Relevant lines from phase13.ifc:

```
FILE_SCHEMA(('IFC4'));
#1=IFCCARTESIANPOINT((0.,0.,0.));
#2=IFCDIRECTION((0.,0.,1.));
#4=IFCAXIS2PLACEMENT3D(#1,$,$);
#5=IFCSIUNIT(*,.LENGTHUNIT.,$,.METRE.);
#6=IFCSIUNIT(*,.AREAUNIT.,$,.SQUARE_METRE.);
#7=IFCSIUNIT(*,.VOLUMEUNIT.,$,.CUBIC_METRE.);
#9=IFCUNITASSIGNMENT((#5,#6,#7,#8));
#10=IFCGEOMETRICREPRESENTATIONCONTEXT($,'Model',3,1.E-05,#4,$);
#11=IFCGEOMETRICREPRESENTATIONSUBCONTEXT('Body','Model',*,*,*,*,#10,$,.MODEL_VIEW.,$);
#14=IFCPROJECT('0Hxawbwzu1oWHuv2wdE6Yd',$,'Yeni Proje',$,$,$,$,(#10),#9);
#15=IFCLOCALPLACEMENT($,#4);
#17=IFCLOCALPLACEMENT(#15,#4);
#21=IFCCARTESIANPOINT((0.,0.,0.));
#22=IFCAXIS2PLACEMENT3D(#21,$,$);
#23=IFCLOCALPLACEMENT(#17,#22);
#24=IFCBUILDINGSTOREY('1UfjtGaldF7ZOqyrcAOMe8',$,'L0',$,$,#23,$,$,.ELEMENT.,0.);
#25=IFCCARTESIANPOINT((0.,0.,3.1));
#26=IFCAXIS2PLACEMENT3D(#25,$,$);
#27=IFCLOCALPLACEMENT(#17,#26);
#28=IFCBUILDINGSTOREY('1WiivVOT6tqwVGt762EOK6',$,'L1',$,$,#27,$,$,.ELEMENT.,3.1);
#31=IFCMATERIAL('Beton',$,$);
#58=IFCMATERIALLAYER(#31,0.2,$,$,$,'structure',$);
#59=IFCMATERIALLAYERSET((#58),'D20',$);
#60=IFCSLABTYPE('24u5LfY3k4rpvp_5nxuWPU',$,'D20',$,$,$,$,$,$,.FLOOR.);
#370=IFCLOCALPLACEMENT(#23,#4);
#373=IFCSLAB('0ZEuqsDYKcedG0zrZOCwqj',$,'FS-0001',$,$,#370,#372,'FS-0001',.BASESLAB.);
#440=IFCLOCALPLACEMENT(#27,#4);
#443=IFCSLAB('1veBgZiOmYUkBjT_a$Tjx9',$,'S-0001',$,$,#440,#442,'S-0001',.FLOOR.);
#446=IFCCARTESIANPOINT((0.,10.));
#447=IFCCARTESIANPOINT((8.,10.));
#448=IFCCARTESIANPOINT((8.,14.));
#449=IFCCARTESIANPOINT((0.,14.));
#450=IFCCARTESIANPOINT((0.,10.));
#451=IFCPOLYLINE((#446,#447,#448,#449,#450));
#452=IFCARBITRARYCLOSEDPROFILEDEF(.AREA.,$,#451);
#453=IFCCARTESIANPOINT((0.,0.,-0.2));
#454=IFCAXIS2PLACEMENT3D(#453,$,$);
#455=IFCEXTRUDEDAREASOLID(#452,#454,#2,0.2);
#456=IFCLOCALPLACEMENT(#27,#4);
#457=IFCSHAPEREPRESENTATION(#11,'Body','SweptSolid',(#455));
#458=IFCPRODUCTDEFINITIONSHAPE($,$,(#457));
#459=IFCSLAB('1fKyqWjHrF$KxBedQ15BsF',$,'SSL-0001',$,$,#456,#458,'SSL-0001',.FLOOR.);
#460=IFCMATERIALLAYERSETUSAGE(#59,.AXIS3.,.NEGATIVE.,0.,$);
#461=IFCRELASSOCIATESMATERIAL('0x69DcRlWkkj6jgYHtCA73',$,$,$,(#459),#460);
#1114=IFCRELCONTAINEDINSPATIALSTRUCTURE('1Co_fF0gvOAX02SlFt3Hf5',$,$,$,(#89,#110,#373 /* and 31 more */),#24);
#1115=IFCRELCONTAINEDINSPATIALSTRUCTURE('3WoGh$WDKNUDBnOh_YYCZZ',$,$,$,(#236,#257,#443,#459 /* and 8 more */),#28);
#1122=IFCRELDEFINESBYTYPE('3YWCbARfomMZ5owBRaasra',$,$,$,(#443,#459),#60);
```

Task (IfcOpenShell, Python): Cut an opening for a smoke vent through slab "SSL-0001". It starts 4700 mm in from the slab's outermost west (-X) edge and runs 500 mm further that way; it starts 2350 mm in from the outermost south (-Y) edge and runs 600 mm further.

```python
import numpy as np
import ifcopenshell
import ifcopenshell.api.feature
import ifcopenshell.api.geometry
import ifcopenshell.api.root
import ifcopenshell.geom
import ifcopenshell.util.placement
import ifcopenshell.util.representation
import ifcopenshell.util.shape
import ifcopenshell.util.unit

model = ifcopenshell.open("phase13.ifc")
unit_scale = ifcopenshell.util.unit.calculate_unit_scale(model)
settings = ifcopenshell.geom.settings()


def volume(element):
    """Net volume in cubic metres, openings subtracted."""
    shape = ifcopenshell.geom.create_shape(settings, element)
    return ifcopenshell.util.shape.get_volume(shape.geometry)


slab = model.by_guid("1fKyqWjHrF$KxBedQ15BsF")
before = volume(slab)

# Extent in the slab's own axes, in metres. The edges named are its -X and -Y sides.
slab_shape = ifcopenshell.geom.create_shape(settings, slab)
vertices = ifcopenshell.util.shape.get_vertices(slab_shape.geometry)
x_min, y_min, bottom = vertices.min(axis=0)
top = vertices[:, 2].max()

opening = ifcopenshell.api.root.create_entity(model, ifc_class="IfcOpeningElement", name="Smoke vent opening", predefined_type="OPENING")
context = ifcopenshell.util.representation.get_context(model, "Model", "Body", "MODEL_VIEW")
width, depth = 0.5, 0.6
outline = [(0.0, 0.0), (width, 0.0), (width, depth), (0.0, depth), (0.0, 0.0)]
# Overshoot both faces by 50 mm so the cut is clean.
shape = ifcopenshell.api.geometry.add_slab_representation(
    model, context=context, depth=top - bottom + 0.1, polyline=outline
)
ifcopenshell.api.geometry.assign_representation(model, product=opening, representation=shape)

matrix = ifcopenshell.util.placement.get_local_placement(slab.ObjectPlacement)
matrix[:, 3] = matrix @ np.append(np.array([x_min + 4.7, y_min + 2.35, bottom - 0.05]) / unit_scale, 1.0)
ifcopenshell.api.geometry.edit_object_placement(model, product=opening, matrix=matrix, is_si=False)
ifcopenshell.api.feature.add_feature(model, feature=opening, element=slab)

after = volume(slab)

print(f"slab volume {before:.3f} -> {after:.3f} m3")

model.write("phase13-out.ifc")
```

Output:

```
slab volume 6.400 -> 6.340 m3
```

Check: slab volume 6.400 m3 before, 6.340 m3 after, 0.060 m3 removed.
